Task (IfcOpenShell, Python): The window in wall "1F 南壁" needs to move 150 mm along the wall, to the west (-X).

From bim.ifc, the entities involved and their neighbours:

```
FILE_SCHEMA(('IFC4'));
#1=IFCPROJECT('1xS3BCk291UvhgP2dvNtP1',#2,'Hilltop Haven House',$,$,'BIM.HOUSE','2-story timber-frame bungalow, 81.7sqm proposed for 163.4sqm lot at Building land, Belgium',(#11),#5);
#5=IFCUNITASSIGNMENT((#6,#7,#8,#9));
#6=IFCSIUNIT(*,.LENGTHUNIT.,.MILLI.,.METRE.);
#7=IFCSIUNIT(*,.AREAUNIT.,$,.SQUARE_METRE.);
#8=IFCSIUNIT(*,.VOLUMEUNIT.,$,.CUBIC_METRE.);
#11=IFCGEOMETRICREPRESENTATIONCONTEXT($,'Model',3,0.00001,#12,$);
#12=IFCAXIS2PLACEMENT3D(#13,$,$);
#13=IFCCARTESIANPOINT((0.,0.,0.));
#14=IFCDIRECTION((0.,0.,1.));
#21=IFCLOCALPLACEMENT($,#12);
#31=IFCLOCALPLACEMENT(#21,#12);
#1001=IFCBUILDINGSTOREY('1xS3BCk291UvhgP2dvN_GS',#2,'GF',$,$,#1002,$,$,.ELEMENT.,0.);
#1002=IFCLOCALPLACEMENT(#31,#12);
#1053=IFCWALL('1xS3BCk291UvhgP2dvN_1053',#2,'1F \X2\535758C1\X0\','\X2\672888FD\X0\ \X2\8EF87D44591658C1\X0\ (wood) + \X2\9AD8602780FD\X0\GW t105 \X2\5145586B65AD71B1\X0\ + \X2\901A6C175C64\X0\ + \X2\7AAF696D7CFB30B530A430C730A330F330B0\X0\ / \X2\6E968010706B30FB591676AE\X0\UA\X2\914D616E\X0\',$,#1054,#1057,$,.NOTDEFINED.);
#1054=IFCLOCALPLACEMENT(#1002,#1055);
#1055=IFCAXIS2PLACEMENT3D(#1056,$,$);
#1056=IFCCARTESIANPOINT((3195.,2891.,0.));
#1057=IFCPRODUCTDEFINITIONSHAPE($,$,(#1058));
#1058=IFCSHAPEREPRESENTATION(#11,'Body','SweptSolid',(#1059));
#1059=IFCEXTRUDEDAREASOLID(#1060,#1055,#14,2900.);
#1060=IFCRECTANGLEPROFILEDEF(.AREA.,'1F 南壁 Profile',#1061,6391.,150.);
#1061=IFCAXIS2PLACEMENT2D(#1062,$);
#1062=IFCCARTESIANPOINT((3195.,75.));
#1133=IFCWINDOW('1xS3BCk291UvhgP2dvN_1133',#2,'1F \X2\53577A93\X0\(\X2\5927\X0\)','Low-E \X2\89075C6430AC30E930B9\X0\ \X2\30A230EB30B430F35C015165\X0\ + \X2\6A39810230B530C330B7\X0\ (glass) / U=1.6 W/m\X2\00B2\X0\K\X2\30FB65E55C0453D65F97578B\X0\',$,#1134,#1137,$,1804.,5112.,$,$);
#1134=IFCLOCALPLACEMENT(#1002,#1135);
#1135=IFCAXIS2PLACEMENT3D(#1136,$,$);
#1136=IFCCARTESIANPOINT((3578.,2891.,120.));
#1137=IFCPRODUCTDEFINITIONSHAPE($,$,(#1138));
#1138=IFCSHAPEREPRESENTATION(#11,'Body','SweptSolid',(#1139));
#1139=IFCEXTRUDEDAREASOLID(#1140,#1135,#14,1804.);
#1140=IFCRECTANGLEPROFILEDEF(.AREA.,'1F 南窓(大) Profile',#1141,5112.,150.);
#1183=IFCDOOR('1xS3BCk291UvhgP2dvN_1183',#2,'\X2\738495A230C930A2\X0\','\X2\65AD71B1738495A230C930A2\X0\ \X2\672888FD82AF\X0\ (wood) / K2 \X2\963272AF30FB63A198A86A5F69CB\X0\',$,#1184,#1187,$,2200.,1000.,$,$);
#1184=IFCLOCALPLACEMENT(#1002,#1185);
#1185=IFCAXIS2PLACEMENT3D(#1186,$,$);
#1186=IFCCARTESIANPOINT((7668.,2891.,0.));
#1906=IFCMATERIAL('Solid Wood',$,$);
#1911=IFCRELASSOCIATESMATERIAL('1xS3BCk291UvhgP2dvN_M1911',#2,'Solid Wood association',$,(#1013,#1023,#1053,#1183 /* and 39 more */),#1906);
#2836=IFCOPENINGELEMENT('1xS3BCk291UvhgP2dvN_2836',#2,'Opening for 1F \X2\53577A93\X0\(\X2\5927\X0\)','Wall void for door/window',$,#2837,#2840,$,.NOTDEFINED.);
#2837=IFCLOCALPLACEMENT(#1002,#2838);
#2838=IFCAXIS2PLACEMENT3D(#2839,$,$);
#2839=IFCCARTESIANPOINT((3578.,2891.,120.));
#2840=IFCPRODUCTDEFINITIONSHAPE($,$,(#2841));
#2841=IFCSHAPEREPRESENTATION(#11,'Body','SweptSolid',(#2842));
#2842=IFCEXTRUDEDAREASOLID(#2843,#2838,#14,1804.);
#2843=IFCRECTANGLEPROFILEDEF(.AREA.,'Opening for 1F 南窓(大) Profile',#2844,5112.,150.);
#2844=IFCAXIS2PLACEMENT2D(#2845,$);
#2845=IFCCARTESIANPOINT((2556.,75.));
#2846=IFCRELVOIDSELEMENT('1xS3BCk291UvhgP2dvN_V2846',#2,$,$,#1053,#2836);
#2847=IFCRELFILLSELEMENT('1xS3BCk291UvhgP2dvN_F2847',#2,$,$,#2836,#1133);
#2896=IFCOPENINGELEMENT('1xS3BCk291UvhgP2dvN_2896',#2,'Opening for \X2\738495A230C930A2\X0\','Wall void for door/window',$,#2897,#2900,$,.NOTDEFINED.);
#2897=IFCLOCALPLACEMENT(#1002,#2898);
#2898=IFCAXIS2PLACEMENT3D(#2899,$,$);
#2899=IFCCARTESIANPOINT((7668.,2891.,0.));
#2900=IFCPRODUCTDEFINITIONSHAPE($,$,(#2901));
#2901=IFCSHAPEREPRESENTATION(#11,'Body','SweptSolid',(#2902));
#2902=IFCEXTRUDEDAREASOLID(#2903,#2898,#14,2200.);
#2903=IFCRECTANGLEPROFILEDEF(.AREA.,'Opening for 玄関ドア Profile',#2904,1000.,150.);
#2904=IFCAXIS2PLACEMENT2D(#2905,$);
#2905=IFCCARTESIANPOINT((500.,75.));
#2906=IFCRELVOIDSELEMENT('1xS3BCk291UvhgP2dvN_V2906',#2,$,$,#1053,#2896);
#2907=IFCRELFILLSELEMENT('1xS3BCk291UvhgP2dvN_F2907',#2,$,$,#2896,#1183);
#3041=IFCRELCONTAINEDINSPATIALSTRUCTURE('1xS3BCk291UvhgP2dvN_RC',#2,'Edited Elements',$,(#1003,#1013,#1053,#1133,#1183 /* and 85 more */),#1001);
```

```python
import ifcopenshell
import ifcopenshell.api.geometry
import ifcopenshell.util.placement

model = ifcopenshell.open("bim.ifc")

window = model.by_guid("1xS3BCk291UvhgP2dvN_1133")
opening = window.FillsVoids[0].RelatingOpeningElement
wall = opening.VoidsElements[0].RelatingBuildingElement

wall_matrix = ifcopenshell.util.placement.get_local_placement(wall.ObjectPlacement)
shift = wall_matrix[:3, 0] * -150.0
before = ifcopenshell.util.placement.get_local_placement(window.ObjectPlacement)[:3, 3].copy()

# The window is not placed relative to its opening, so move both.
for product in (opening, window):
    matrix = ifcopenshell.util.placement.get_local_placement(product.ObjectPlacement)
    matrix[:3, 3] += shift
    ifcopenshell.api.geometry.edit_object_placement(model, product=product, matrix=matrix, is_si=False)

after = ifcopenshell.util.placement.get_local_placement(window.ObjectPlacement)[:3, 3]
print("window moved by", (after - before).round(3) + 0.0)

model.write("bim_v2.ifc")
```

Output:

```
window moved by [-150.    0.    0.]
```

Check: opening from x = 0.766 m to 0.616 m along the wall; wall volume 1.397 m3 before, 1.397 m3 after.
